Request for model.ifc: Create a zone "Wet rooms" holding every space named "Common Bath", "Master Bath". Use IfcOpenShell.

First a look at what the model holds.

```python
import ifcopenshell

model = ifcopenshell.open("model.ifc")
print(model.schema)
seen = {}
for space in model.by_type("IfcSpace"):
    seen[space.LongName] = seen.get(space.LongName, 0) + 1
for name, count in sorted(seen.items(), key=str):
    print(count, "x", name)
print("zones:", [z.Name for z in model.by_type("IfcZone")][:20])
```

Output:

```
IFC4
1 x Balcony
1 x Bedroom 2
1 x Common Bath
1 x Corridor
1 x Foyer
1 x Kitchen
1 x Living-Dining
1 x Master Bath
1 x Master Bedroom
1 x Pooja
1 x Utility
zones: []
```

```python
import ifcopenshell
import ifcopenshell.api.group
import ifcopenshell.api.root

model = ifcopenshell.open("model.ifc")

names = {"Common Bath", "Master Bath"}
spaces = [s for s in model.by_type("IfcSpace") if s.LongName in names]

zone = ifcopenshell.api.root.create_entity(model, ifc_class="IfcZone", name="Wet rooms")
ifcopenshell.api.group.assign_group(model, products=spaces, group=zone)
print(len(spaces), "spaces in", zone.Name)

model.write("model-out.ifc")
```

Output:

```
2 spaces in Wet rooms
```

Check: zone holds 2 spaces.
